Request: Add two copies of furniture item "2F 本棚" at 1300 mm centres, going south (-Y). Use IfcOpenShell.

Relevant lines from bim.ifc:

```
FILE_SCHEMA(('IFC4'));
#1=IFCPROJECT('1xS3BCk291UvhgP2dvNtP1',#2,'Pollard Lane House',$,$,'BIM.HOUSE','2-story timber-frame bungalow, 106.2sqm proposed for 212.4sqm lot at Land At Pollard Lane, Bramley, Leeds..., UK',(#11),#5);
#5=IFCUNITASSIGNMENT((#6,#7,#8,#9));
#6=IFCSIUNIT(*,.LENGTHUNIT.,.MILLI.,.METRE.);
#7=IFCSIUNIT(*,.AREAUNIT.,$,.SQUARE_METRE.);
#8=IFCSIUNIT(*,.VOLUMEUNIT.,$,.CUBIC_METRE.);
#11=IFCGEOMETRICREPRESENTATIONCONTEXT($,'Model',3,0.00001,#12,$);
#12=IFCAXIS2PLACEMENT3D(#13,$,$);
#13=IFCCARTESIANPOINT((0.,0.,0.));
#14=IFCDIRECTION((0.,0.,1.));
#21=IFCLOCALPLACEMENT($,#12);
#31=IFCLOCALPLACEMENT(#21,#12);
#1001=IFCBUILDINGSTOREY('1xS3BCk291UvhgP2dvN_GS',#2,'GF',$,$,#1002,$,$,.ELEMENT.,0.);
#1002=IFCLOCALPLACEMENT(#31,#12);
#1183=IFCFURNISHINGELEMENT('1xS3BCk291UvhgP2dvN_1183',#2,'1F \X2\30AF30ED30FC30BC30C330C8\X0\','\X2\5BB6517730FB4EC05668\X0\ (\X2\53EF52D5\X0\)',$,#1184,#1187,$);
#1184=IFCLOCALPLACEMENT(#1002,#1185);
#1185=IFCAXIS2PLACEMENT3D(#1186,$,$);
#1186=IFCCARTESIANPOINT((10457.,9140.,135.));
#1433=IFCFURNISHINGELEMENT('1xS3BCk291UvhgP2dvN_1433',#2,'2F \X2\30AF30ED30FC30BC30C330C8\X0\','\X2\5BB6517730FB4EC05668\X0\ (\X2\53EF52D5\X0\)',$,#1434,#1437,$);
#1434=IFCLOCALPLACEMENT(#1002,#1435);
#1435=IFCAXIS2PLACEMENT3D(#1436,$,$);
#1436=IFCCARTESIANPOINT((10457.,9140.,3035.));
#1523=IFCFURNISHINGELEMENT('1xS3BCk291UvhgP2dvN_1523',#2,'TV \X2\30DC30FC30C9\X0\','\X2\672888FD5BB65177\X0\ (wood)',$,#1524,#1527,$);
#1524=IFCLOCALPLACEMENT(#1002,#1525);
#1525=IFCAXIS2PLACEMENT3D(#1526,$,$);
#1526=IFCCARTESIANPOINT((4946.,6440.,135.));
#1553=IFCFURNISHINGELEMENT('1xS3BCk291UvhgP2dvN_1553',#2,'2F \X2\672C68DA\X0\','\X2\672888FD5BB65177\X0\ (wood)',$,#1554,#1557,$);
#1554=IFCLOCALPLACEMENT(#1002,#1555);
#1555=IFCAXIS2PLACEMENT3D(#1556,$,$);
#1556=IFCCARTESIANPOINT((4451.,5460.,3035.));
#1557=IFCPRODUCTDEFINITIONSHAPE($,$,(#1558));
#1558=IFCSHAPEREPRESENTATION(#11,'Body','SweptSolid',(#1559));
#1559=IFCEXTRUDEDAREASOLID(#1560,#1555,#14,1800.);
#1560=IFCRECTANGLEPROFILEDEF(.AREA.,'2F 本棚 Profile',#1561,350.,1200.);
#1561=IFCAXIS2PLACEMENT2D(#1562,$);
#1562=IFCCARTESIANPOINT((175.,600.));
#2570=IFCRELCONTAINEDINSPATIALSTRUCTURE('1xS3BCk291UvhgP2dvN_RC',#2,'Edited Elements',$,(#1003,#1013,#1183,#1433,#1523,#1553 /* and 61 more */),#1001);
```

```python
import numpy as np
import ifcopenshell
import ifcopenshell.api.geometry
import ifcopenshell.api.root
import ifcopenshell.util.element
import ifcopenshell.util.placement
import ifcopenshell.util.unit

model = ifcopenshell.open("bim.ifc")
unit_scale = ifcopenshell.util.unit.calculate_unit_scale(model)


def reuse_history(source, copy):
    """copy_class also copies each property set's owner history, people and application; keep the originals."""
    for rel in copy.IsDefinedBy:
        if rel.is_a("IfcRelDefinesByProperties") and (history := rel.RelatingPropertyDefinition.OwnerHistory):
            rel.RelatingPropertyDefinition.OwnerHistory = source.OwnerHistory
            ifcopenshell.util.element.remove_deep2(model, history)


source = model.by_id(1553)
base = ifcopenshell.util.placement.get_local_placement(source.ObjectPlacement)
step = np.array([0.0, -1.0, 0.0]) * 1.3 / unit_scale

for i in range(1, 3):
    copy = ifcopenshell.api.root.copy_class(model, product=source)
    copy.Representation = ifcopenshell.util.element.copy_deep(
        model, source.Representation, exclude=["IfcGeometricRepresentationContext", "IfcRepresentationMap"]
    )
    reuse_history(source, copy)
    matrix = base.copy()
    matrix[:3, 3] += i * step
    print("added at", matrix[:3, 3].round(3) + 0.0)
    ifcopenshell.api.geometry.edit_object_placement(model, product=copy, matrix=matrix, is_si=False)

model.write("bim_edited.ifc")
```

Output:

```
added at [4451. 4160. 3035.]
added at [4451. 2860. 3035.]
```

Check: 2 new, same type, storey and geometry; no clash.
